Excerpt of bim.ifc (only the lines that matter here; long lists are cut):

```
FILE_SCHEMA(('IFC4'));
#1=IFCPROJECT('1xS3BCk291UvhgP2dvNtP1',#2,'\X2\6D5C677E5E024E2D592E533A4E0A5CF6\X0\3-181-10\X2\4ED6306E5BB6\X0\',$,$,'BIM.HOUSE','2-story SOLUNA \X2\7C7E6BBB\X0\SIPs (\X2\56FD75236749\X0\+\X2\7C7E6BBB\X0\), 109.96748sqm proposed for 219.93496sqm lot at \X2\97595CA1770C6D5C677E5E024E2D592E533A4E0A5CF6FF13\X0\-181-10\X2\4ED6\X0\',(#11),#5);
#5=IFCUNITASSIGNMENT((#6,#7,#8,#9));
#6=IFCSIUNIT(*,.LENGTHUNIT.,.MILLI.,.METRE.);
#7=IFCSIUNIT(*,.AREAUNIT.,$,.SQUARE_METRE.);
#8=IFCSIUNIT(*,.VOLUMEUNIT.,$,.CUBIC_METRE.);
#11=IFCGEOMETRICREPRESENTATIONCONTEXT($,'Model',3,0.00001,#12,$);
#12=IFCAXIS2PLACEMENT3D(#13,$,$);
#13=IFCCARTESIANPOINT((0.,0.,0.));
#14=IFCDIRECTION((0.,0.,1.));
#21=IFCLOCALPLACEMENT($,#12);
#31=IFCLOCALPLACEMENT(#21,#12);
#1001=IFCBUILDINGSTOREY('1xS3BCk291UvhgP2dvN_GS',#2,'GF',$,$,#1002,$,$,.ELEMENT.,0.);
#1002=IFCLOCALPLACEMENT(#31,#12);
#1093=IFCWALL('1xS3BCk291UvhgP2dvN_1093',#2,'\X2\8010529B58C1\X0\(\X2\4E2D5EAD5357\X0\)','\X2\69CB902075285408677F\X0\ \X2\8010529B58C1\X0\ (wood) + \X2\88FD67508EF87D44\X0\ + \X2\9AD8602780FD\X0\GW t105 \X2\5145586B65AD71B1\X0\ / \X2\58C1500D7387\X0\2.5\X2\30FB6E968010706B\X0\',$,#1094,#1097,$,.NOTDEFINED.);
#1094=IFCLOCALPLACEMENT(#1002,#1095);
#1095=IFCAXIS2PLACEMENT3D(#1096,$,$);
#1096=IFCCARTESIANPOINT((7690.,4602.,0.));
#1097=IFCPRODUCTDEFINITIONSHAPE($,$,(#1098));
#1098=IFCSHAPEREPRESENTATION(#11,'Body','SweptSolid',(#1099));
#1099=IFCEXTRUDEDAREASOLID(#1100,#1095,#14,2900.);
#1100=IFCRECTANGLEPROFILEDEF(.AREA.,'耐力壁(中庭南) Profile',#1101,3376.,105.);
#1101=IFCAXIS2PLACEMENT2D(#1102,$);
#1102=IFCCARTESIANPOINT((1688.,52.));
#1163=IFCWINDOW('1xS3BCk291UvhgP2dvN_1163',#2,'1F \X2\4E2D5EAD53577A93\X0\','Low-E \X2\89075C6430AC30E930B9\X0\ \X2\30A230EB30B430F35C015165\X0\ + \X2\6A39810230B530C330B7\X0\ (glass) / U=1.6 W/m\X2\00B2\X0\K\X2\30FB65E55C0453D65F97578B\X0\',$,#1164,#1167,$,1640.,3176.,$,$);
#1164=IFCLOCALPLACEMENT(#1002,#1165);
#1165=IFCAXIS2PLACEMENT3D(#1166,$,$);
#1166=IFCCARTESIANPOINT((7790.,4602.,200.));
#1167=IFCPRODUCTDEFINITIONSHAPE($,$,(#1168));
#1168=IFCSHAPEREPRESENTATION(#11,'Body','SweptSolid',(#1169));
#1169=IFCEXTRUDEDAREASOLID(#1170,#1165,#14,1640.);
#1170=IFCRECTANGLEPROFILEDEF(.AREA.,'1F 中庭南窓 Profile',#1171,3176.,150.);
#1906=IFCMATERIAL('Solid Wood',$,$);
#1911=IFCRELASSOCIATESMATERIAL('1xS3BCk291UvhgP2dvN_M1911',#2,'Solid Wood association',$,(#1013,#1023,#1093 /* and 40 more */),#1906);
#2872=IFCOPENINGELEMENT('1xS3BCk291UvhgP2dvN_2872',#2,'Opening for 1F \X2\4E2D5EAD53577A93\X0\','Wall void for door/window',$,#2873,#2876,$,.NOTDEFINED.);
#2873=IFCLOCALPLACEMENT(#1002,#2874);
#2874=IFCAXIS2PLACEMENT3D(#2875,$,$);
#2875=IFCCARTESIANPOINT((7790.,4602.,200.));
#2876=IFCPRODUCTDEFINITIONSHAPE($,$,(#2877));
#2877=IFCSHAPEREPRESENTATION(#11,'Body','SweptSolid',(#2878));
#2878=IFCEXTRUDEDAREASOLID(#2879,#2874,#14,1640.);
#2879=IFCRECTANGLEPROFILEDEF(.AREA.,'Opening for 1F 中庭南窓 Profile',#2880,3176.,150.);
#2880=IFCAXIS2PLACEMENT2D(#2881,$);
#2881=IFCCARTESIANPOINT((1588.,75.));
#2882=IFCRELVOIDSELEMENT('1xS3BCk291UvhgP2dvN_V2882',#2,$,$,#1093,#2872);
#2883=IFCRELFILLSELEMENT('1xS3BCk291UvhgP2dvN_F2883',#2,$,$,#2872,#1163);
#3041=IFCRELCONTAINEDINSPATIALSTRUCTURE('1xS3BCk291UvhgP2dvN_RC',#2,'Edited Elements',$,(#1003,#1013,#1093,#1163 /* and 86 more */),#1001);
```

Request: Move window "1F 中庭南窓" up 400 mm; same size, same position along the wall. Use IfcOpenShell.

```python
import numpy as np
import ifcopenshell
import ifcopenshell.api.geometry
import ifcopenshell.util.placement
import ifcopenshell.util.unit

model = ifcopenshell.open("bim.ifc")
unit_scale = ifcopenshell.util.unit.calculate_unit_scale(model)

window = model.by_guid("1xS3BCk291UvhgP2dvN_1163")
opening = window.FillsVoids[0].RelatingOpeningElement
dz = 0.4 / unit_scale

shift = np.array([0.0, 0.0, dz])
# The window is not placed relative to its opening, so move both.
for product in (opening, window):
    matrix = ifcopenshell.util.placement.get_local_placement(product.ObjectPlacement)
    matrix[:3, 3] += shift
    ifcopenshell.api.geometry.edit_object_placement(model, product=product, matrix=matrix, is_si=False)

print(f"moved by {dz * unit_scale:+.3f} m")

model.write("bim_updated.ifc")
```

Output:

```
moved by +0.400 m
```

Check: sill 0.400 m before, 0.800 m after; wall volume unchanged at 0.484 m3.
